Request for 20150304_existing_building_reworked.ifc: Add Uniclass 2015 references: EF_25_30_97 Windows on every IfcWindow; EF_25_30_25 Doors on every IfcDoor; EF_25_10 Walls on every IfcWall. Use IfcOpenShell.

First a look at what the model holds.

```python
import ifcopenshell

model = ifcopenshell.open("20150304_existing_building_reworked.ifc")
print(model.schema)
print("classifications:", [c.Name for c in model.by_type("IfcClassification")])
for ifc_class in ("IfcDoor", "IfcRoof", "IfcStair", "IfcWall", "IfcWindow"):
    print(ifc_class, len(model.by_type(ifc_class)))
```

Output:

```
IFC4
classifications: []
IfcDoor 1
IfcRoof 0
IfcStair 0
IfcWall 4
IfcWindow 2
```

```python
import ifcopenshell
import ifcopenshell.api.classification

model = ifcopenshell.open("20150304_existing_building_reworked.ifc")

system = ifcopenshell.api.classification.add_classification(model, classification="Uniclass 2015")

codes = {
    "IfcWindow": ("EF_25_30_97", "Windows"),
    "IfcDoor": ("EF_25_30_25", "Doors"),
    "IfcWall": ("EF_25_10", "Walls"),
}
for ifc_class, (code, name) in codes.items():
    products = model.by_type(ifc_class)
    ifcopenshell.api.classification.add_reference(
        model, products=products, classification=system, identification=code, name=name
    )
    print(code, len(products))

model.write("20150304_existing_building_reworked-out.ifc")
```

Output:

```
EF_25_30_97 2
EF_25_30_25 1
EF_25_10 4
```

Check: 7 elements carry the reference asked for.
